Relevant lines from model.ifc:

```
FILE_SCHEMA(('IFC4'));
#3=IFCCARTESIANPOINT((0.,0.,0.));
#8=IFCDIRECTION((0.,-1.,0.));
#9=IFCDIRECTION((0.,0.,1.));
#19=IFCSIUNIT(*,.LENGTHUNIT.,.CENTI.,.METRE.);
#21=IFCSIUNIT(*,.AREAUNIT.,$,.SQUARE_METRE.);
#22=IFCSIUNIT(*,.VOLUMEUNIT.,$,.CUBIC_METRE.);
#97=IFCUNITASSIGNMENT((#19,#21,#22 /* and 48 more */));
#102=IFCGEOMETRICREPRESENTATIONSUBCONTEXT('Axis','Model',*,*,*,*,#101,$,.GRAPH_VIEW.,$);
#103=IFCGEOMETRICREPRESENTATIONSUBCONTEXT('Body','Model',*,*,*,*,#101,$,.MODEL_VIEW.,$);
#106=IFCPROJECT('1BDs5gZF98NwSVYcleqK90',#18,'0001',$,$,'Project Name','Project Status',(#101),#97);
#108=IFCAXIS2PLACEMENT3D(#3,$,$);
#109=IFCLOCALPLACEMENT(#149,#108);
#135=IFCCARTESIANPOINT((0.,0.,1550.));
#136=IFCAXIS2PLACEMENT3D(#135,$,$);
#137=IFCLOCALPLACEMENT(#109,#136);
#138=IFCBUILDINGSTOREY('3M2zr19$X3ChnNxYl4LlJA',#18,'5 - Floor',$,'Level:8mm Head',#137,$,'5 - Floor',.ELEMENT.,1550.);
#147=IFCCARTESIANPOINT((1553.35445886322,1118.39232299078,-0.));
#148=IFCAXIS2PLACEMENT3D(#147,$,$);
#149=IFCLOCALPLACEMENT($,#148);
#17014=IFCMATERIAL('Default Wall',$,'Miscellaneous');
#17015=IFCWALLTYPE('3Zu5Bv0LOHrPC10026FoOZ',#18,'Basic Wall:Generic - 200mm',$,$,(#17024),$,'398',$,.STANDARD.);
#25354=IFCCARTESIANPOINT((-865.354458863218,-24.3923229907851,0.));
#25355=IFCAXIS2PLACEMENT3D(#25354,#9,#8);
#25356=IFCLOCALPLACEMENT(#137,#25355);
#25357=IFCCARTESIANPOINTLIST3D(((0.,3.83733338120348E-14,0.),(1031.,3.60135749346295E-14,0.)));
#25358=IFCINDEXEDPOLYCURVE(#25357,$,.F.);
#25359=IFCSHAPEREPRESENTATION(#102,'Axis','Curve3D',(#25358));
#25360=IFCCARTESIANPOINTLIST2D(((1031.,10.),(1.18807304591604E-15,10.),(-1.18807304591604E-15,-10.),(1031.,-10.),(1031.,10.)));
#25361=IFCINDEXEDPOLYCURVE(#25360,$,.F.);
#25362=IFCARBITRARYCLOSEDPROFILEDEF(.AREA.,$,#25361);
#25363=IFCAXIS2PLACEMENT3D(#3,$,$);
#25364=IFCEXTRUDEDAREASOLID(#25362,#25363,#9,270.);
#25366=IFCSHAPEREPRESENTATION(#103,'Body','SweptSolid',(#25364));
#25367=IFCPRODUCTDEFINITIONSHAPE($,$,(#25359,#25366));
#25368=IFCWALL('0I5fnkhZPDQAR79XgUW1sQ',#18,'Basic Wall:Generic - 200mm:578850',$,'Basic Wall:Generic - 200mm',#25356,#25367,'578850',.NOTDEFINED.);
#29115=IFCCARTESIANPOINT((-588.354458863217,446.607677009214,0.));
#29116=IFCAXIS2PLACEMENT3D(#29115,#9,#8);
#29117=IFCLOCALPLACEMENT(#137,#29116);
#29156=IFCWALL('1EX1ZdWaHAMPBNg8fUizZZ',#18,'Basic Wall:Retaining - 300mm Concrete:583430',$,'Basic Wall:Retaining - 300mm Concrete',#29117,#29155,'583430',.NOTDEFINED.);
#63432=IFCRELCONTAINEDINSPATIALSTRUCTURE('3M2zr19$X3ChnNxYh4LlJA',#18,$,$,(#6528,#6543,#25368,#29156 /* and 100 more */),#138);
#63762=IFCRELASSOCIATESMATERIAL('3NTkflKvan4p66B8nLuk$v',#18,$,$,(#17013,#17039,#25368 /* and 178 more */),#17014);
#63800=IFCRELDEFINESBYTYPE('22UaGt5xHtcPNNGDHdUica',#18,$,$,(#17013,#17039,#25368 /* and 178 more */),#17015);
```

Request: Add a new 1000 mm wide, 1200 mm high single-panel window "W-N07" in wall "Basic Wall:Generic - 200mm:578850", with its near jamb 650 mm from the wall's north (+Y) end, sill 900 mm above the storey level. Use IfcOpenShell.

```python
import numpy as np
import ifcopenshell
import ifcopenshell.api.feature
import ifcopenshell.api.geometry
import ifcopenshell.api.root
import ifcopenshell.api.spatial
import ifcopenshell.geom
import ifcopenshell.util.element
import ifcopenshell.util.placement
import ifcopenshell.util.representation
import ifcopenshell.util.shape
import ifcopenshell.util.unit

model = ifcopenshell.open("model.ifc")
unit_scale = ifcopenshell.util.unit.calculate_unit_scale(model)
settings = ifcopenshell.geom.settings()


def volume(element):
    """Net volume in cubic metres, openings subtracted."""
    shape = ifcopenshell.geom.create_shape(settings, element)
    return ifcopenshell.util.shape.get_volume(shape.geometry)


wall = model.by_guid("0I5fnkhZPDQAR79XgUW1sQ")
storey = ifcopenshell.util.element.get_container(wall, ifc_class="IfcBuildingStorey")
context = ifcopenshell.util.representation.get_context(model, "Model", "Body", "MODEL_VIEW")
before = volume(wall)

width, height, from_end, sill = 1, 1.2, 0.65, 0.9  # metres

# The wall runs along its own X axis, and the end named is its -X end.
wall_shape = ifcopenshell.geom.create_shape(settings, wall)
x, y, z = ifcopenshell.util.shape.get_vertices(wall_shape.geometry).T
start = x.min() + from_end
face, thickness = float(y.min()), float(y.max() - y.min())
wall_matrix = ifcopenshell.util.placement.get_local_placement(wall.ObjectPlacement)
level = ifcopenshell.util.placement.get_local_placement(storey.ObjectPlacement)[2, 3]


def in_wall(x, y):
    """Placement at x, y metres in the wall's axes, at sill height."""
    matrix = wall_matrix.copy()
    matrix[:, 3] = wall_matrix @ np.array([x / unit_scale, y / unit_scale, 0.0, 1.0])
    matrix[2, 3] = level + sill / unit_scale
    return matrix


# Opening: a box that overshoots both wall faces by 50 mm.
opening = ifcopenshell.api.root.create_entity(model, ifc_class="IfcOpeningElement", predefined_type="OPENING")
box = ifcopenshell.api.geometry.add_wall_representation(
    model, context=context, length=width, height=height, thickness=thickness + 0.1
)
ifcopenshell.api.geometry.assign_representation(model, product=opening, representation=box)
ifcopenshell.api.geometry.edit_object_placement(model, product=opening, matrix=in_wall(start, face - 0.05), is_si=False)
ifcopenshell.api.feature.add_feature(model, feature=opening, element=wall)

window = ifcopenshell.api.root.create_entity(model, ifc_class="IfcWindow", name="W-N07", predefined_type="WINDOW")
window.OverallWidth, window.OverallHeight = width / unit_scale, height / unit_scale
window.PartitioningType = "SINGLE_PANEL"
body = ifcopenshell.api.geometry.add_window_representation(
    model,
    context=context,
    overall_width=window.OverallWidth,
    overall_height=window.OverallHeight,
    partition_type="SINGLE_PANEL",
)
ifcopenshell.api.geometry.assign_representation(model, product=window, representation=body)
ifcopenshell.api.spatial.assign_container(model, products=[window], relating_structure=storey)
ifcopenshell.api.feature.add_filling(model, opening=opening, element=window)

# Centre the window in the wall's thickness.
ifcopenshell.api.geometry.edit_object_placement(model, product=window, matrix=in_wall(start, face), is_si=False)
window_shape = ifcopenshell.geom.create_shape(settings, window)
depth = ifcopenshell.util.shape.get_vertices(window_shape.geometry)[:, 1]
offset = face + thickness / 2 - (depth.min() + depth.max()) / 2
ifcopenshell.api.geometry.edit_object_placement(model, product=window, matrix=in_wall(start, offset), is_si=False)

after = volume(wall)

print(f"wall volume {before:.3f} -> {after:.3f} m3")

model.write("model_edited.ifc")
```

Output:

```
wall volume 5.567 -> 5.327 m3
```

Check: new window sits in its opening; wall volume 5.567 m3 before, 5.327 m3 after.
